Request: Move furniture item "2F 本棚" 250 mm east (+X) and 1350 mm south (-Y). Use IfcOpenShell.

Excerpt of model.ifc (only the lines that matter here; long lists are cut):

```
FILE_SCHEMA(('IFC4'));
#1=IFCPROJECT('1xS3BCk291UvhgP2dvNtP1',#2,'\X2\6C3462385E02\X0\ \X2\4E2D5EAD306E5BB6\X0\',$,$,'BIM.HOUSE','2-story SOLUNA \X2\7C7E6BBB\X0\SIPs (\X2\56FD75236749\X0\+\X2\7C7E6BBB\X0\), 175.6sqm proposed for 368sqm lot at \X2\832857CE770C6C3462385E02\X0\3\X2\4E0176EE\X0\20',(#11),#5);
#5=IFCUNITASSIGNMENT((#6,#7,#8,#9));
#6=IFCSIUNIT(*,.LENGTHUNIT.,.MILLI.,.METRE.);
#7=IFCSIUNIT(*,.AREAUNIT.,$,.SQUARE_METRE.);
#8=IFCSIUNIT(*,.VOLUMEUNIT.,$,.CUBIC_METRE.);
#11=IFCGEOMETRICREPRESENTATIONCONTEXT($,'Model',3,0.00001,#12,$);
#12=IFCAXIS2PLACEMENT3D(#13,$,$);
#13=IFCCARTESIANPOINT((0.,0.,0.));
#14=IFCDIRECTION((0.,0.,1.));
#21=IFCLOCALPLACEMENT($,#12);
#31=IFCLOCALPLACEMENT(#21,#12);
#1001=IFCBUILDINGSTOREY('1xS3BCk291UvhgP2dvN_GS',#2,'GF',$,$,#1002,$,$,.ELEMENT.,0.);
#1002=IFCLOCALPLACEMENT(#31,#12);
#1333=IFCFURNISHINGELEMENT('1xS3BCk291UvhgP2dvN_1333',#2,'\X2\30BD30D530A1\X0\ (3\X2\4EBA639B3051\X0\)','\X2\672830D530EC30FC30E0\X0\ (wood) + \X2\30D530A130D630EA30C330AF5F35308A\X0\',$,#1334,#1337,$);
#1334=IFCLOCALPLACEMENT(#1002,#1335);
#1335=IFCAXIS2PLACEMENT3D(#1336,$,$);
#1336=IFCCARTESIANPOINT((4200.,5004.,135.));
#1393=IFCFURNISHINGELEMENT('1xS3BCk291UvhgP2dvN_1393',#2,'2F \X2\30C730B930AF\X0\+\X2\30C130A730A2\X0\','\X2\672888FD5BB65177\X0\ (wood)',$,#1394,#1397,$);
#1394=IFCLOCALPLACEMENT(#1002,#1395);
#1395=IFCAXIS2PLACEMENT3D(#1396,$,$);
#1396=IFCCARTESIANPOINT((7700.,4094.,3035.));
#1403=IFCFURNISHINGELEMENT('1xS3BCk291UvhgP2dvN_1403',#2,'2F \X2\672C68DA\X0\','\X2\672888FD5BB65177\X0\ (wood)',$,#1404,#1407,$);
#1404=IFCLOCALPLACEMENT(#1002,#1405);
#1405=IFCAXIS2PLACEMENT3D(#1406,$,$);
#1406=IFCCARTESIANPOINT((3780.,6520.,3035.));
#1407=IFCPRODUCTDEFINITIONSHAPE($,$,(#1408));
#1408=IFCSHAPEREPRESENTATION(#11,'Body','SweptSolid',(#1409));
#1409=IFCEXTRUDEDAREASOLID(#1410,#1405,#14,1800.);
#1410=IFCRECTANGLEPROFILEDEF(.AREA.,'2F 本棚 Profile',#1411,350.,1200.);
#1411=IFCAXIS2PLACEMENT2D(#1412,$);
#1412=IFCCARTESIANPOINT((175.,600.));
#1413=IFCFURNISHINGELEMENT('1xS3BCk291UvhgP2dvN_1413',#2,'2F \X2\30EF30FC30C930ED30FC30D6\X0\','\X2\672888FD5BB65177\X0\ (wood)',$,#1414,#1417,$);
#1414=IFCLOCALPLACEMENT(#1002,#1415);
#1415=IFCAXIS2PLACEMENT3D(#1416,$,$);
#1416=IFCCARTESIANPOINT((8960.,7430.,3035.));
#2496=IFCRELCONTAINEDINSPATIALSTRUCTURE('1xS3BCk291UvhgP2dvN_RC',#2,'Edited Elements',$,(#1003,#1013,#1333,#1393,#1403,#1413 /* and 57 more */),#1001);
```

```python
import ifcopenshell
import ifcopenshell.api.geometry
import ifcopenshell.util.placement
import ifcopenshell.util.unit

model = ifcopenshell.open("model.ifc")
unit_scale = ifcopenshell.util.unit.calculate_unit_scale(model)

item = model.by_id(1403)
matrix = ifcopenshell.util.placement.get_local_placement(item.ObjectPlacement)
matrix[0, 3] += 0.25 / unit_scale
matrix[1, 3] -= 1.35 / unit_scale
ifcopenshell.api.geometry.edit_object_placement(model, product=item, matrix=matrix, is_si=False)

print(ifcopenshell.util.placement.get_local_placement(item.ObjectPlacement).round(3) + 0.0)

model.write("model-out.ifc")
```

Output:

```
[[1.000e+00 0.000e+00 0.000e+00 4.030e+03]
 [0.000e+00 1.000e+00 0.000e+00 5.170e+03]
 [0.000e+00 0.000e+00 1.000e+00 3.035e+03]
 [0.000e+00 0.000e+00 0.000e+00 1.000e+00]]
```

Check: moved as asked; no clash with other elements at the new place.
